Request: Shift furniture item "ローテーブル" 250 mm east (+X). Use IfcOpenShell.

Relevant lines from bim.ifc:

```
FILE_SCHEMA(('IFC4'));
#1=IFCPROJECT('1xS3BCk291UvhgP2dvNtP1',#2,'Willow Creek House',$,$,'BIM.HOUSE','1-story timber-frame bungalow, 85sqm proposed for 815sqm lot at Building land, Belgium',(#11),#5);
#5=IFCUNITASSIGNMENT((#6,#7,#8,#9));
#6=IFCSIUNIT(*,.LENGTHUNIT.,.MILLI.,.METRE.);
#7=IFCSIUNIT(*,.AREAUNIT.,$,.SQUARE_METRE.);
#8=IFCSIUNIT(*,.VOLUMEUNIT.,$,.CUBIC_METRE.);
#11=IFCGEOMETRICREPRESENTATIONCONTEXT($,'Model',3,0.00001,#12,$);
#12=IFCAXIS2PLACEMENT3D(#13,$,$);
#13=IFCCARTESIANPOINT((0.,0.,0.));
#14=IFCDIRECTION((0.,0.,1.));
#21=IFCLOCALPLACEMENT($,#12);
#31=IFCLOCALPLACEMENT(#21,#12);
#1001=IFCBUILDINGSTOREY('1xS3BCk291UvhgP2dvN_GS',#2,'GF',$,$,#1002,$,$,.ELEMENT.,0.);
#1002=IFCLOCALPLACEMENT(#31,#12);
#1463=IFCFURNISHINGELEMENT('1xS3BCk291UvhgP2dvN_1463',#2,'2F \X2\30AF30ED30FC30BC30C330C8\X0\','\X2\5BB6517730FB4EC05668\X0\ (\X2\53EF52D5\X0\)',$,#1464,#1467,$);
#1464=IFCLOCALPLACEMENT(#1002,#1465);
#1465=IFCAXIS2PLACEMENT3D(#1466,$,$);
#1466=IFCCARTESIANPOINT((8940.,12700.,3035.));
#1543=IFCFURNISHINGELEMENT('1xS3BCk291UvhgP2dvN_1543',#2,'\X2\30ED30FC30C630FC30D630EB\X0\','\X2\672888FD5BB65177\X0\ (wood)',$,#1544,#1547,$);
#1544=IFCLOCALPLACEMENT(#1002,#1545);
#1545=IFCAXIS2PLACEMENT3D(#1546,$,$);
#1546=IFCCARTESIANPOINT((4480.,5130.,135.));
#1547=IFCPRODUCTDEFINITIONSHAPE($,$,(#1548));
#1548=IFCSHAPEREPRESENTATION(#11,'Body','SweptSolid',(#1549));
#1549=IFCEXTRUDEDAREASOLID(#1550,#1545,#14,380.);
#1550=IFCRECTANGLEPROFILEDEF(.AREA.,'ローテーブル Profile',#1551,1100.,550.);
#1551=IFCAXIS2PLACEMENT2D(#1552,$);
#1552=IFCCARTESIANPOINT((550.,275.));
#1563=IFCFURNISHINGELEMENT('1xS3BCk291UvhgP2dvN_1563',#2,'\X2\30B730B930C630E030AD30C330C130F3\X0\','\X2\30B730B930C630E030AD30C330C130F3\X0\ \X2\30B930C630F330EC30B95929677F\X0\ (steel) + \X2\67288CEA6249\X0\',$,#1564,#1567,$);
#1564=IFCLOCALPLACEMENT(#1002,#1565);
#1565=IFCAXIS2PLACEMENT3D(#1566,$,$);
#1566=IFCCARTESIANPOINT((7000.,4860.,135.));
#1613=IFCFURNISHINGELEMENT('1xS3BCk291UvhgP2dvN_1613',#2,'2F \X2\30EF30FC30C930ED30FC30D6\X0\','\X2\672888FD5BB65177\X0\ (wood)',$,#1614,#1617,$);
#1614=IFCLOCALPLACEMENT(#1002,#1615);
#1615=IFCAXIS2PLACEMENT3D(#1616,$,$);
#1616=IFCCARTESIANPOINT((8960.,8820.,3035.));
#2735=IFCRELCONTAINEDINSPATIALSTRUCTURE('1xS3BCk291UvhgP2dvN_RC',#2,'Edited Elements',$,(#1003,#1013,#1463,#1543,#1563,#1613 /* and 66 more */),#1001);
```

```python
import ifcopenshell
import ifcopenshell.api.geometry
import ifcopenshell.util.placement
import ifcopenshell.util.unit

model = ifcopenshell.open("bim.ifc")
unit_scale = ifcopenshell.util.unit.calculate_unit_scale(model)

item = model.by_guid("1xS3BCk291UvhgP2dvN_1543")
matrix = ifcopenshell.util.placement.get_local_placement(item.ObjectPlacement)
matrix[0, 3] += 0.25 / unit_scale
ifcopenshell.api.geometry.edit_object_placement(model, product=item, matrix=matrix, is_si=False)

print(ifcopenshell.util.placement.get_local_placement(item.ObjectPlacement).round(3) + 0.0)

model.write("bim_rev.ifc")
```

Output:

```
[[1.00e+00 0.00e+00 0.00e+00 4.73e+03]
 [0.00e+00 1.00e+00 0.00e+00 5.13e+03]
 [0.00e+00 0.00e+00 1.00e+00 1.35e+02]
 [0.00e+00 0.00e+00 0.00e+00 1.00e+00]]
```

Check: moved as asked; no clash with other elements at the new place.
